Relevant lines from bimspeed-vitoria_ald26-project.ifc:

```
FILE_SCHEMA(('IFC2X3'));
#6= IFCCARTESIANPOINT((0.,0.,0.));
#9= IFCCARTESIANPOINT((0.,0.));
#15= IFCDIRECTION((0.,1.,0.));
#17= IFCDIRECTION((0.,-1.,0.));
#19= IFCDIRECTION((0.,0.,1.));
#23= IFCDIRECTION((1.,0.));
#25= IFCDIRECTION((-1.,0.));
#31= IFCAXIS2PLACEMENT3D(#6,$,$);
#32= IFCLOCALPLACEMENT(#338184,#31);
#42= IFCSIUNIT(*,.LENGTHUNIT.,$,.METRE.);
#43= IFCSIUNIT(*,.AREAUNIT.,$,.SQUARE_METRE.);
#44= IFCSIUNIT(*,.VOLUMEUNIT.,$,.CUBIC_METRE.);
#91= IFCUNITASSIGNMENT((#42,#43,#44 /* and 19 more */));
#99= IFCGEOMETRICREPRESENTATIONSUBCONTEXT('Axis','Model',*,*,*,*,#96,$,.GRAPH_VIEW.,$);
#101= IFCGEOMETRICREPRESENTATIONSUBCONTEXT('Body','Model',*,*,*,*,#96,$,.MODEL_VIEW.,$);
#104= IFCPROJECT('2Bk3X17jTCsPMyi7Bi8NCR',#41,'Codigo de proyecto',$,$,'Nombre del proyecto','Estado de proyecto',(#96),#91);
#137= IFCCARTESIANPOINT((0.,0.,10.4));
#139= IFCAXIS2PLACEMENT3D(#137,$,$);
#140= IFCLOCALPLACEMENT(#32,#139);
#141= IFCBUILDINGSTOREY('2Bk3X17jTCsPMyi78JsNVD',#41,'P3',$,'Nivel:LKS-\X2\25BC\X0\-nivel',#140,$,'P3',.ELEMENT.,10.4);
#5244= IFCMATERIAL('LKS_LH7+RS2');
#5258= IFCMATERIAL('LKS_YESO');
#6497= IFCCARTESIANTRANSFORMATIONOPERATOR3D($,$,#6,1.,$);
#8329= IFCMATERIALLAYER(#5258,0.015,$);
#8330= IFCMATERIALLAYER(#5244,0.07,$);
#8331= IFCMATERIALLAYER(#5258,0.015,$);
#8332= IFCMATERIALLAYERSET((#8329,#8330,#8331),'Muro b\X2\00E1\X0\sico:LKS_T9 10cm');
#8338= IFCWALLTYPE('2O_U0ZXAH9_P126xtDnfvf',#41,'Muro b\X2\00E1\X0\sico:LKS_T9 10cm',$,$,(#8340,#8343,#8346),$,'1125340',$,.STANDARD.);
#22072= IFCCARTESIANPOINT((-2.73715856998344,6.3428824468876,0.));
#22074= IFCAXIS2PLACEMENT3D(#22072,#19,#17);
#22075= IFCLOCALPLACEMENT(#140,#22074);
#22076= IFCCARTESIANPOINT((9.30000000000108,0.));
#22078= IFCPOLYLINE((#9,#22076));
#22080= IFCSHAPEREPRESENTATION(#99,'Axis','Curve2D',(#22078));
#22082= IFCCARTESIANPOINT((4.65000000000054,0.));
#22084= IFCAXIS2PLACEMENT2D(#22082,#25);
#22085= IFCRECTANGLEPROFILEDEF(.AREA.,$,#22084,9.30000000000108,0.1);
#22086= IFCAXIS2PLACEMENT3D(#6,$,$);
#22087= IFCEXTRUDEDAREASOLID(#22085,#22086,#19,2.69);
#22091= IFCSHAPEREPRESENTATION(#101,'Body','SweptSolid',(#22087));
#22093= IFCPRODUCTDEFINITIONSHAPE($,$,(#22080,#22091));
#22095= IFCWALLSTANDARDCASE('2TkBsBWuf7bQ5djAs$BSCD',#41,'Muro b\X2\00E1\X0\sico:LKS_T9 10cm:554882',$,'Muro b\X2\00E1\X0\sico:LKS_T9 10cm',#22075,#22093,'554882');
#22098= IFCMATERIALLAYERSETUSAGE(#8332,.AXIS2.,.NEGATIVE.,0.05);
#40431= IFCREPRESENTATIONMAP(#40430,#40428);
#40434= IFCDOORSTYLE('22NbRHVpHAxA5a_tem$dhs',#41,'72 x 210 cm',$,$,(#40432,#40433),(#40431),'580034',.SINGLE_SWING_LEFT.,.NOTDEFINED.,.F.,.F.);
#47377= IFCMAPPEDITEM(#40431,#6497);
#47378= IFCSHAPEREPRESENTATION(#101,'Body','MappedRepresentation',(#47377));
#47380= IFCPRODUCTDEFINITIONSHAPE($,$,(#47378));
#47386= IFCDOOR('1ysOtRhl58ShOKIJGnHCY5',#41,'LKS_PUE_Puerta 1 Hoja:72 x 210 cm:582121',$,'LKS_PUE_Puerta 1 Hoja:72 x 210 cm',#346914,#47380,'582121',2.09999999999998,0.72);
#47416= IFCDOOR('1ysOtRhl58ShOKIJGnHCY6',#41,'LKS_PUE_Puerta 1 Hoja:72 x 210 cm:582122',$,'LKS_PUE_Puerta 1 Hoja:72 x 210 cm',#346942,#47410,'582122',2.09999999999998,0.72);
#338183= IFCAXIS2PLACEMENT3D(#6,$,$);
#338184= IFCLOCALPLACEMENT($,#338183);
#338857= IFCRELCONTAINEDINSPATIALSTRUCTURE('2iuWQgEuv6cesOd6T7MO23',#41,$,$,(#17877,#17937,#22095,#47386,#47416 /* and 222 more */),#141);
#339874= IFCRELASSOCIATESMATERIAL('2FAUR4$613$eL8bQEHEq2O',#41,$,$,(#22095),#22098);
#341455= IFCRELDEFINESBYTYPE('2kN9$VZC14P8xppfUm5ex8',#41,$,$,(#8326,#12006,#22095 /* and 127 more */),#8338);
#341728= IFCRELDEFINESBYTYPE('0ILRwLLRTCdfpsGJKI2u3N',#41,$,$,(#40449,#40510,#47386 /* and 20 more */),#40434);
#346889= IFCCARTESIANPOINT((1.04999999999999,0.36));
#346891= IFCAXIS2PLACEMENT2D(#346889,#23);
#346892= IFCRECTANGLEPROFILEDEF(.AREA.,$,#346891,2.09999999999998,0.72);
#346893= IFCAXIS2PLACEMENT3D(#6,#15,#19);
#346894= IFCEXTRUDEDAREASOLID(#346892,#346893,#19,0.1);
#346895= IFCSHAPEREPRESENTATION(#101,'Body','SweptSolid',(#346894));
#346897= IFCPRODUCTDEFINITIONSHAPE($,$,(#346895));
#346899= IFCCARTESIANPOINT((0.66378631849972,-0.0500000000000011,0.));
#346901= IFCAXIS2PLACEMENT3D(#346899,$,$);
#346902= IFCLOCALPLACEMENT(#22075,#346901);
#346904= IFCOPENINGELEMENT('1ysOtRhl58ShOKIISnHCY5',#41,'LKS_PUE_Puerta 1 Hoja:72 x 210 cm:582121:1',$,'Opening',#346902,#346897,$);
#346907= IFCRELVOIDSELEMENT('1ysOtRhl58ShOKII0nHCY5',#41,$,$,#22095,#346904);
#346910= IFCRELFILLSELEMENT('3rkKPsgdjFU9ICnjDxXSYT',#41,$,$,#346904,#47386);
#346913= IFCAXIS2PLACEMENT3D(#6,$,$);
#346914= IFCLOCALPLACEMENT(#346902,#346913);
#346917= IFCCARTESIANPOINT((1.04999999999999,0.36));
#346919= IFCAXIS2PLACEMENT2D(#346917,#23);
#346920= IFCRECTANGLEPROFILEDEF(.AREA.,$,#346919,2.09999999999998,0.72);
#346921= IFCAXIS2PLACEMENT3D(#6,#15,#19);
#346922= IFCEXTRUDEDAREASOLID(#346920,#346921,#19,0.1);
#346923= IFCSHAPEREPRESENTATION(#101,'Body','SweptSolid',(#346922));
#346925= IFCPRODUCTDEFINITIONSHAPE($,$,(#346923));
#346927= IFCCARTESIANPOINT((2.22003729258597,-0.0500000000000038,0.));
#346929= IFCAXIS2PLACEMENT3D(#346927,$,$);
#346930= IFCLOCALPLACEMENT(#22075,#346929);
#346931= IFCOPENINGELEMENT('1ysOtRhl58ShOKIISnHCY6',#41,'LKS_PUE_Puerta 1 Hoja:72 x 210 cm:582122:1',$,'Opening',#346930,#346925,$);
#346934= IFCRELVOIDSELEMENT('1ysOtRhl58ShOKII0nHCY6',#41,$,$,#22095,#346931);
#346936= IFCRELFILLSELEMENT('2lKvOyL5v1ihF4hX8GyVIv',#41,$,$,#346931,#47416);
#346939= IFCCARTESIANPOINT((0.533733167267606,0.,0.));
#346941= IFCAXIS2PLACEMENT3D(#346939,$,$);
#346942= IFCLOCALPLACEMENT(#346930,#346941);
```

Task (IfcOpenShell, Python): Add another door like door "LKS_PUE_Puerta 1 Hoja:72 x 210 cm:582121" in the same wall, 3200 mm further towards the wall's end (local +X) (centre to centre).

```python
import ifcopenshell
import ifcopenshell.api.feature
import ifcopenshell.api.geometry
import ifcopenshell.api.root
import ifcopenshell.geom
import ifcopenshell.util.element
import ifcopenshell.util.placement
import ifcopenshell.util.shape

model = ifcopenshell.open("bimspeed-vitoria_ald26-project.ifc")
settings = ifcopenshell.geom.settings()


def volume(element):
    """Net volume in cubic metres, openings subtracted."""
    shape = ifcopenshell.geom.create_shape(settings, element)
    return ifcopenshell.util.shape.get_volume(shape.geometry)


def reuse_history(source, copy):
    """copy_class also copies each property set's owner history, people and application; keep the originals."""
    for rel in copy.IsDefinedBy:
        if rel.is_a("IfcRelDefinesByProperties") and (history := rel.RelatingPropertyDefinition.OwnerHistory):
            rel.RelatingPropertyDefinition.OwnerHistory = source.OwnerHistory
            ifcopenshell.util.element.remove_deep2(model, history)


door = model.by_id(47386)
opening = door.FillsVoids[0].RelatingOpeningElement
wall = opening.VoidsElements[0].RelatingBuildingElement
before = volume(wall)
shift = ifcopenshell.util.placement.get_local_placement(wall.ObjectPlacement)[:3, 0] * 3.2

# copy_class copies the void relationship, type, container and properties, but no geometry.
new_opening = ifcopenshell.api.root.copy_class(model, product=opening)
new_opening.Representation = ifcopenshell.util.element.copy_deep(
    model, opening.Representation, exclude=["IfcGeometricRepresentationContext", "IfcRepresentationMap"]
)
new_opening.Name = "LKS_PUE_Puerta 1 Hoja:72 x 210 cm"
new_door = ifcopenshell.api.root.copy_class(model, product=door)
new_door.Representation = ifcopenshell.util.element.copy_deep(
    model, door.Representation, exclude=["IfcGeometricRepresentationContext", "IfcRepresentationMap"]
)
new_door.Name = "LKS_PUE_Puerta 1 Hoja:72 x 210 cm"
new_door.Tag = None
reuse_history(door, new_door)
fills = ifcopenshell.api.feature.add_filling(model, opening=new_opening, element=new_door)
fills.OwnerHistory = new_door.OwnerHistory  # required in IFC2X3

for old, new in ((opening, new_opening), (door, new_door)):
    matrix = ifcopenshell.util.placement.get_local_placement(old.ObjectPlacement)
    matrix[:3, 3] += shift
    ifcopenshell.api.geometry.edit_object_placement(model, product=new, matrix=matrix, is_si=False)

after = volume(wall)

print(f"wall volume {before:.3f} -> {after:.3f} m3")

model.write("bimspeed-vitoria_ald26-project_edited.ifc")
```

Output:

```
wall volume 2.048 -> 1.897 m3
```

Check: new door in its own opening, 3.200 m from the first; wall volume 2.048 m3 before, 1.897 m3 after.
